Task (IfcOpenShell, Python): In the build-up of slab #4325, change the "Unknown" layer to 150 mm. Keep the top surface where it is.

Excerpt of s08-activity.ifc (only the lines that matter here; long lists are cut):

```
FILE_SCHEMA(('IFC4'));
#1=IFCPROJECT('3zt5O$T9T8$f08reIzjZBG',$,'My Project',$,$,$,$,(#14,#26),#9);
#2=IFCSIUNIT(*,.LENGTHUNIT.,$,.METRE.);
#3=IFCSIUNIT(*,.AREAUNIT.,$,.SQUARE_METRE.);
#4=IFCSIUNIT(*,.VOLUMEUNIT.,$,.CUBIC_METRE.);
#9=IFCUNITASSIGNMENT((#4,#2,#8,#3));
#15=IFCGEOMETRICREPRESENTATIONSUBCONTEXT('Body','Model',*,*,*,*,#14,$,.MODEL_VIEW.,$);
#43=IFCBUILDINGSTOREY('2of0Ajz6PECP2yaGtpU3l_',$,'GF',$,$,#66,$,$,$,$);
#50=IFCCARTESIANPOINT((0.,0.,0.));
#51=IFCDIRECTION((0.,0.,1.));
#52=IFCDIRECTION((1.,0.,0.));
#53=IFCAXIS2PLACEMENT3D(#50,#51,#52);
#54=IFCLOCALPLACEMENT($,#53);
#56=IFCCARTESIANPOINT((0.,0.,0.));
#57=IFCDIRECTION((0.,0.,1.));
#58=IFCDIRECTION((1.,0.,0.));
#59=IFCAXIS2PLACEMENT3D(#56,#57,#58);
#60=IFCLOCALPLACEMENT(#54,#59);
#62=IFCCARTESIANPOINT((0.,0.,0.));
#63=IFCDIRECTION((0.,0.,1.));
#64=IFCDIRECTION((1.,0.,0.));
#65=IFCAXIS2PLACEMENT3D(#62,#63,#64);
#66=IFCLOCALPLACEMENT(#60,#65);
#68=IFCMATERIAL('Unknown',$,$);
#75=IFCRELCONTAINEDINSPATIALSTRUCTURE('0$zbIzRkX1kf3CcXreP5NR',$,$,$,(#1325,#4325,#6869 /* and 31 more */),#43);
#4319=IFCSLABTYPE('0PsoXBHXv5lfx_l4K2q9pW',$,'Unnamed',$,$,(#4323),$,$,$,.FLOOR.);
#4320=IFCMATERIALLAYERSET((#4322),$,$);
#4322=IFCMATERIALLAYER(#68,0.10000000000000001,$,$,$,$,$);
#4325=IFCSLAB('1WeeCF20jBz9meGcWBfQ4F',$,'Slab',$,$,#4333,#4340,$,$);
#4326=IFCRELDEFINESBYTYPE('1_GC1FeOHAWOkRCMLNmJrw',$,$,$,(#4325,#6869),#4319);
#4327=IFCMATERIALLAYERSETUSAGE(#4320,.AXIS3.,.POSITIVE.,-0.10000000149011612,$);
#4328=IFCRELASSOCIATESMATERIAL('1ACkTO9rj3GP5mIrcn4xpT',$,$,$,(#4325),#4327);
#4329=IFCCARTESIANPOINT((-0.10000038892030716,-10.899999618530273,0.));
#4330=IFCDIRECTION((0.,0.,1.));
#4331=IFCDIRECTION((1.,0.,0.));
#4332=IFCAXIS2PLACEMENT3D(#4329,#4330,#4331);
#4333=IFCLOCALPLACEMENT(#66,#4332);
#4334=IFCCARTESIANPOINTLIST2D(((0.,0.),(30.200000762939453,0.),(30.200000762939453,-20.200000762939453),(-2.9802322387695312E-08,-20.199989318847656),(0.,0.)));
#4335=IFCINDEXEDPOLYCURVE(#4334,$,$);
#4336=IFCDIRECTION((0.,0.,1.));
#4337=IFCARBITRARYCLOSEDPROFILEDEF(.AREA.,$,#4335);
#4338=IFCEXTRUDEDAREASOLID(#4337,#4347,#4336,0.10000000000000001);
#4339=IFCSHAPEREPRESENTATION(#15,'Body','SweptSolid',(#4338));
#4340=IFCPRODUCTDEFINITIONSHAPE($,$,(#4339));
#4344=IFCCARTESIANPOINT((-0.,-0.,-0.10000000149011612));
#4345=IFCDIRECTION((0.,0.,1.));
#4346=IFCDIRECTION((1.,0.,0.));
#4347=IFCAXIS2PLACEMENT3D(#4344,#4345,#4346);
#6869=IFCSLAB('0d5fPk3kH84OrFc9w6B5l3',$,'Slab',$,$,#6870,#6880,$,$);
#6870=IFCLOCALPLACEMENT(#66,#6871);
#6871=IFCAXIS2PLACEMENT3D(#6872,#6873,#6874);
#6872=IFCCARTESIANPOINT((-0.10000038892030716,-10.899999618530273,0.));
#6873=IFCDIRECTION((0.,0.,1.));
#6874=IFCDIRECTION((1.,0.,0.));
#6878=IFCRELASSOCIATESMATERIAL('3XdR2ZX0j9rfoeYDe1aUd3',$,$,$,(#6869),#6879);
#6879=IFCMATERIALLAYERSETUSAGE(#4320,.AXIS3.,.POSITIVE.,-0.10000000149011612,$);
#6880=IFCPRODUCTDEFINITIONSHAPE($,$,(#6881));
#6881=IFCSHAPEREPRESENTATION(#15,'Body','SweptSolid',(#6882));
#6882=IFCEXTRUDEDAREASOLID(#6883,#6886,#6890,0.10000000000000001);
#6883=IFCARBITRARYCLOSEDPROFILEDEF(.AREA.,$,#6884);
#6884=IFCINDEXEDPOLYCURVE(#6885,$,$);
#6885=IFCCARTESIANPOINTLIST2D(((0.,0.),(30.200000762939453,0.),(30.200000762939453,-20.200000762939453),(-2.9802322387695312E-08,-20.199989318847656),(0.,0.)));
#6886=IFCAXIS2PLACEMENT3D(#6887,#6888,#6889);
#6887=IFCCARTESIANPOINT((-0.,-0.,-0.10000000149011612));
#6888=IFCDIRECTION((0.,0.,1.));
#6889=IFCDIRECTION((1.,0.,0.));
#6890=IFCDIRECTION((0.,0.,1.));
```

```python
import ifcopenshell
import ifcopenshell.util.element
import ifcopenshell.util.representation
import ifcopenshell.util.unit

model = ifcopenshell.open("s08-activity.ifc")
unit_scale = ifcopenshell.util.unit.calculate_unit_scale(model)

layer_set = model.by_id(4320)
layer = next(l for l in layer_set.MaterialLayers if l.Material and l.Material.Name == "Unknown")
change = 0.15 / unit_scale - layer.LayerThickness
layer.LayerThickness += change

# The layer set is shared, so every slab that uses it gets the new thickness.
slabs = [e for e in ifcopenshell.util.element.get_elements_by_material(model, layer_set) if e.is_a("IfcSlab")]
for slab in sorted(slabs, key=lambda e: e.id()):
    body = ifcopenshell.util.representation.get_representation(slab, "Model", "Body")
    solid = body.Items[0]
    old_depth = solid.Depth
    solid.Depth += change
    # Extruded upwards: lower the start of the extrusion so the top stays.
    x, y, z = solid.Position.Location.Coordinates
    solid.Position.Location = model.createIfcCartesianPoint((x, y, z - change))
    print(slab.id(), f"{old_depth:g} -> {solid.Depth:g}")

# The layers are counted up from the underside, which has moved.
for usage in {ifcopenshell.util.element.get_material(slab) for slab in slabs}:
    usage.OffsetFromReferenceLine -= change

model.write("s08-activity_updated.ifc")
```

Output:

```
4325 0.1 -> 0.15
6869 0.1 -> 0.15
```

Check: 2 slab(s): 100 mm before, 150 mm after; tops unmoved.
